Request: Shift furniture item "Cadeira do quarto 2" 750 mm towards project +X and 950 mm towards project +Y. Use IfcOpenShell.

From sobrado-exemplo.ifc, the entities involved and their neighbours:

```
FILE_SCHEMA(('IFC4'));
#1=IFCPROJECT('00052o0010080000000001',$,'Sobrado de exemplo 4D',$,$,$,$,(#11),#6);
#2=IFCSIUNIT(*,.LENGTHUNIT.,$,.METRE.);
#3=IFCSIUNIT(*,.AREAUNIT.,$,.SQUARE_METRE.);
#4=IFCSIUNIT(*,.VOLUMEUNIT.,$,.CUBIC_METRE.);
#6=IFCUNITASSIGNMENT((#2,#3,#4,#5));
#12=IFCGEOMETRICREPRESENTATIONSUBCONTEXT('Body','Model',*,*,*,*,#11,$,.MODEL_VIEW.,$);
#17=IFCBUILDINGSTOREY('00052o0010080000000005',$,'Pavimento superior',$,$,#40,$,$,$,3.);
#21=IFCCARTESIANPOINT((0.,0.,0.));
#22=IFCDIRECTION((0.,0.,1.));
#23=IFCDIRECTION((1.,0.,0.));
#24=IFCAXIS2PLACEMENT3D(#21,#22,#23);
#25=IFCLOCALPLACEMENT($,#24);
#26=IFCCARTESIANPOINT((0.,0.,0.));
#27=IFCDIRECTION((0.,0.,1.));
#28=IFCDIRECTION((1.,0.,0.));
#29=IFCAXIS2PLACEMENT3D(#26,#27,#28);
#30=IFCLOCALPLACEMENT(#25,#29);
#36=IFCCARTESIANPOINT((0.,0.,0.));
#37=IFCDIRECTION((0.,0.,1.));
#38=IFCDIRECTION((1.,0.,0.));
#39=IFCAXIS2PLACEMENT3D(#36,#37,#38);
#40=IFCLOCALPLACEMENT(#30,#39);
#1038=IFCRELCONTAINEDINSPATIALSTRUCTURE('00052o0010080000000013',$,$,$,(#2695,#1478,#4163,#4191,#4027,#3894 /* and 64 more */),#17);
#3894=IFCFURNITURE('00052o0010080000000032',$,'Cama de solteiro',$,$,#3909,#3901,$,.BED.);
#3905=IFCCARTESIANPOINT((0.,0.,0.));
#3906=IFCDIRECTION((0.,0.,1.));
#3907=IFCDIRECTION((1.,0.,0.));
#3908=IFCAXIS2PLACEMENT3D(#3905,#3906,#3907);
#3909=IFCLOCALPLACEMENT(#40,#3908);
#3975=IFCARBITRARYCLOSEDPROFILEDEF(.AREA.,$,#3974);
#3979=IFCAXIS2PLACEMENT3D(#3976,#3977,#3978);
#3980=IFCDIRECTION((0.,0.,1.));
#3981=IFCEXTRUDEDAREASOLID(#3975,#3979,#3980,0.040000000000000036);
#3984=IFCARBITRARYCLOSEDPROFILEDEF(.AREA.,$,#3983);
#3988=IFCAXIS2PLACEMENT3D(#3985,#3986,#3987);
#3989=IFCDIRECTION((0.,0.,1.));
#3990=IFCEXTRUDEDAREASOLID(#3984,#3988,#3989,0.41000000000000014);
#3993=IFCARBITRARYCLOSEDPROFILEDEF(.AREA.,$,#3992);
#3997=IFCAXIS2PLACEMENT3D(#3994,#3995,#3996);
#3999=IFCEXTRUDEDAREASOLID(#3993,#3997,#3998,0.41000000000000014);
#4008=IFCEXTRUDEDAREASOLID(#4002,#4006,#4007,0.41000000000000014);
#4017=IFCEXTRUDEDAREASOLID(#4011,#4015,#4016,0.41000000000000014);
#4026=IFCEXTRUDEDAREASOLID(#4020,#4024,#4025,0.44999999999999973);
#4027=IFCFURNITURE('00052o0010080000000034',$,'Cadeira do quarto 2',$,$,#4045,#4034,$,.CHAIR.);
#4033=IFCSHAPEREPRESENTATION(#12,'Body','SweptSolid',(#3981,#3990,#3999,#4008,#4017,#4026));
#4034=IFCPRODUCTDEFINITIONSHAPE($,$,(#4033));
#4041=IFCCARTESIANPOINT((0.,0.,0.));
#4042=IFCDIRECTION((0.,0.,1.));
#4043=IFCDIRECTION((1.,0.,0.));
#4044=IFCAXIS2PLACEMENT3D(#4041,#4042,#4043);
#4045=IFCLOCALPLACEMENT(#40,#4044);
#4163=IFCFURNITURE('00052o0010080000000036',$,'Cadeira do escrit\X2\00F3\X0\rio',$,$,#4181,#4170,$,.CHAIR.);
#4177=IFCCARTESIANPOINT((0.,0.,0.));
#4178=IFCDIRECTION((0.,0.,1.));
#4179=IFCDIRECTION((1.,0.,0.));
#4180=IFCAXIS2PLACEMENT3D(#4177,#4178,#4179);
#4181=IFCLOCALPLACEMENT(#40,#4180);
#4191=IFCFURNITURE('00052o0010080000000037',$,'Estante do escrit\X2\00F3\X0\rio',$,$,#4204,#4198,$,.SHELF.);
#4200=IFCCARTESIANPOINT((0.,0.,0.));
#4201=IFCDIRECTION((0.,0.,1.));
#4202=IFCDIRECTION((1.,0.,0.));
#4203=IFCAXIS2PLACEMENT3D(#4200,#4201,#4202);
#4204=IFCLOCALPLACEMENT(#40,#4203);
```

```python
import ifcopenshell
import ifcopenshell.api.geometry
import ifcopenshell.util.placement
import ifcopenshell.util.unit

model = ifcopenshell.open("sobrado-exemplo.ifc")
unit_scale = ifcopenshell.util.unit.calculate_unit_scale(model)

item = model.by_guid("00052o0010080000000034")
matrix = ifcopenshell.util.placement.get_local_placement(item.ObjectPlacement)
matrix[0, 3] += 0.75 / unit_scale
matrix[1, 3] += 0.95 / unit_scale
ifcopenshell.api.geometry.edit_object_placement(model, product=item, matrix=matrix, is_si=False)

print(ifcopenshell.util.placement.get_local_placement(item.ObjectPlacement).round(3) + 0.0)

model.write("sobrado-exemplo_rev.ifc")
```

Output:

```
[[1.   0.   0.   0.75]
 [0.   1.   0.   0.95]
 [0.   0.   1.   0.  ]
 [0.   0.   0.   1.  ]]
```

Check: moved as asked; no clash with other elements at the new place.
